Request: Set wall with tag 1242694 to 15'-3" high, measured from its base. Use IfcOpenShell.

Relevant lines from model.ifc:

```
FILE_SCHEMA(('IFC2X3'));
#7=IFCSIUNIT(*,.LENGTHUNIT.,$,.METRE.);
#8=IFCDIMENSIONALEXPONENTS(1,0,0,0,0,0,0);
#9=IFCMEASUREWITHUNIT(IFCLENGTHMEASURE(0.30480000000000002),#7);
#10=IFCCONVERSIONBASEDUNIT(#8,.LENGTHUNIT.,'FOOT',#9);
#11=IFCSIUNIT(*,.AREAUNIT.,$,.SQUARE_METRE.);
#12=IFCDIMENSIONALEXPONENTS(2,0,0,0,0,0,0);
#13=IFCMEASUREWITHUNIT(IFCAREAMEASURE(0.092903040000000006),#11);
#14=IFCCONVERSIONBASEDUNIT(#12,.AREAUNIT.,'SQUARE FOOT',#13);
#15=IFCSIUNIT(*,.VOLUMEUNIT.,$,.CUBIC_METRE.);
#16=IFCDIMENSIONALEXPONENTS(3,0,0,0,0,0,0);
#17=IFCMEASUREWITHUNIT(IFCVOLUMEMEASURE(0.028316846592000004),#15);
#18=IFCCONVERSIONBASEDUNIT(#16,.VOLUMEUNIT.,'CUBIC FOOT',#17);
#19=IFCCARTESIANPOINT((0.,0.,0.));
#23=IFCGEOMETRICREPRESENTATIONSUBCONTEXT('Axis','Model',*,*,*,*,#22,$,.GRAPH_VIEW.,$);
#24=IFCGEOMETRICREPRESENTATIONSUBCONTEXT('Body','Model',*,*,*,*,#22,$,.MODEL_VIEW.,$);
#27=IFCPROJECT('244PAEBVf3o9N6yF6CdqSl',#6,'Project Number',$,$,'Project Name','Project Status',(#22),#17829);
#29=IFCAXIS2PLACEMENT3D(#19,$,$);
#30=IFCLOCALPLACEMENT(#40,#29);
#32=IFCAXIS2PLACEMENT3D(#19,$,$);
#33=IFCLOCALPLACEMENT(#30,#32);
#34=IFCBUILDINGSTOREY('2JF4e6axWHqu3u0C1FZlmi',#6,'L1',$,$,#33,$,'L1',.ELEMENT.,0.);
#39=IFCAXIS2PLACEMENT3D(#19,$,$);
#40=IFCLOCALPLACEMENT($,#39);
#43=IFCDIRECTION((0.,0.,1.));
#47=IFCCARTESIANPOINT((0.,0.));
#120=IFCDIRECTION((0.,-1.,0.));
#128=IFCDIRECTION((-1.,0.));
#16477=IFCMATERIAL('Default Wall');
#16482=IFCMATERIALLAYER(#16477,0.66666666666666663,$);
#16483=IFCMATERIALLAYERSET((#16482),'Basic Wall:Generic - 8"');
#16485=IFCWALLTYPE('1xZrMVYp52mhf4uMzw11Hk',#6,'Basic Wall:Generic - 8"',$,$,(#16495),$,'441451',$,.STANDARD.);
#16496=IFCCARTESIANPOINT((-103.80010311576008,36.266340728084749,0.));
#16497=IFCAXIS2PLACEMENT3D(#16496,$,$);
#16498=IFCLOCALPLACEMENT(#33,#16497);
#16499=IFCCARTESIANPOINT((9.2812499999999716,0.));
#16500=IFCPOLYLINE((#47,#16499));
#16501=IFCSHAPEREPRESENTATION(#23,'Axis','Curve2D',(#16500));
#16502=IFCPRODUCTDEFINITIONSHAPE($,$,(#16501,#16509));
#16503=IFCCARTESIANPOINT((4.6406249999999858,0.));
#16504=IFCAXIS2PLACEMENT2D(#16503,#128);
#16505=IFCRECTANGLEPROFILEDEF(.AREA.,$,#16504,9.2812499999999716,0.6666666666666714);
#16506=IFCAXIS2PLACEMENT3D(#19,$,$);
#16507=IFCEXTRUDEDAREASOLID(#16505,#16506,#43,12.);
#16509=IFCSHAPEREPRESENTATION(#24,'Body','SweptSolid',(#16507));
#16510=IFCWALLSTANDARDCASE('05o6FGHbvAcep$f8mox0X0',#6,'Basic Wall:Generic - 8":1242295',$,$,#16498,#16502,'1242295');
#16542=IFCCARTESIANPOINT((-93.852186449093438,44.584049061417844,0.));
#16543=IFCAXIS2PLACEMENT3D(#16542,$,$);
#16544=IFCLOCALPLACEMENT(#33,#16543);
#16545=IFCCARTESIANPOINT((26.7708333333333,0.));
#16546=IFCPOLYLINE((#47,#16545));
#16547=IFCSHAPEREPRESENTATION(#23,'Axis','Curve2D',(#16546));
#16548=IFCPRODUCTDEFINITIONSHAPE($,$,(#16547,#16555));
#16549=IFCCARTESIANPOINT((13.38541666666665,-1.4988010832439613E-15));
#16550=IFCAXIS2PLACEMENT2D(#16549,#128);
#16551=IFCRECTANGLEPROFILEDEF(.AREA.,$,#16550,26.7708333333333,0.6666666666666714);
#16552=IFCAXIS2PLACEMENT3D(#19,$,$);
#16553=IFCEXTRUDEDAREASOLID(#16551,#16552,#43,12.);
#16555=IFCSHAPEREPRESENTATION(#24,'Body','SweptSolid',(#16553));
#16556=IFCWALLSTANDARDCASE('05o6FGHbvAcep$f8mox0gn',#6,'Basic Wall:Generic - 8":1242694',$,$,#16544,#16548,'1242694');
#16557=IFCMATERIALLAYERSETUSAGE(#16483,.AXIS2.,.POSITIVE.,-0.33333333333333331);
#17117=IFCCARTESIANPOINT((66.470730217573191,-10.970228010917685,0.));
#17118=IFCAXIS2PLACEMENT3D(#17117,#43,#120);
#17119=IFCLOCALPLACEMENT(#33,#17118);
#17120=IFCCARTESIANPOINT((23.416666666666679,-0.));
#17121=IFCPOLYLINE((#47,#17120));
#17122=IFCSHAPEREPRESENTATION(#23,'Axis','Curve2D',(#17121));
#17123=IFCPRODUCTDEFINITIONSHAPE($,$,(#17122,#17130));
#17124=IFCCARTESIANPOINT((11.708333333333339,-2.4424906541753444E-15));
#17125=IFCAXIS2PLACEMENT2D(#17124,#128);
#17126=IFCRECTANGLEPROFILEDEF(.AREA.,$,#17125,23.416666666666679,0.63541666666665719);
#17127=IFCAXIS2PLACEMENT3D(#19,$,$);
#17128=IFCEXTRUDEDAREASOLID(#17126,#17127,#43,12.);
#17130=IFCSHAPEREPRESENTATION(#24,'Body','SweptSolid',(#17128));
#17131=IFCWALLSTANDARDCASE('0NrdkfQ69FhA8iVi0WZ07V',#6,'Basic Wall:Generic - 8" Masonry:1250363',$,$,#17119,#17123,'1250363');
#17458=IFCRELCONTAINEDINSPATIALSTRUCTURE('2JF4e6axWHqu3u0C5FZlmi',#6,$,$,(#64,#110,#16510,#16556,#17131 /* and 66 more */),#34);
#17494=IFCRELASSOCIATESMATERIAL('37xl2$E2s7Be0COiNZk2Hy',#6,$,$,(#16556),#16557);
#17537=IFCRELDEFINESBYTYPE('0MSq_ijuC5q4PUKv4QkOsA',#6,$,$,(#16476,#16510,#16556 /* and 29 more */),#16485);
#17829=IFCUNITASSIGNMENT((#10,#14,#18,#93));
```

```python
import ifcopenshell
import ifcopenshell.geom
import ifcopenshell.util.representation
import ifcopenshell.util.shape
import ifcopenshell.util.unit

model = ifcopenshell.open("model.ifc")
unit_scale = ifcopenshell.util.unit.calculate_unit_scale(model)
settings = ifcopenshell.geom.settings()


def volume(element):
    """Net volume in cubic metres, openings subtracted."""
    shape = ifcopenshell.geom.create_shape(settings, element)
    return ifcopenshell.util.shape.get_volume(shape.geometry)


wall = model.by_id(16556)
before = volume(wall)

body = ifcopenshell.util.representation.get_representation(wall, "Model", "Body")
solid = body.Items[0]
old_height = solid.Depth
solid.Depth = 183 * 0.0254 / unit_scale
after = volume(wall)

print(f"height {old_height:g} -> {solid.Depth:g}, volume {before:.3f} -> {after:.3f} m3")

model.write("model_rev.ifc")
```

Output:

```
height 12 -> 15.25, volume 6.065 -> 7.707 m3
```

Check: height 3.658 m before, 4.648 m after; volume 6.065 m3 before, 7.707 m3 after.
